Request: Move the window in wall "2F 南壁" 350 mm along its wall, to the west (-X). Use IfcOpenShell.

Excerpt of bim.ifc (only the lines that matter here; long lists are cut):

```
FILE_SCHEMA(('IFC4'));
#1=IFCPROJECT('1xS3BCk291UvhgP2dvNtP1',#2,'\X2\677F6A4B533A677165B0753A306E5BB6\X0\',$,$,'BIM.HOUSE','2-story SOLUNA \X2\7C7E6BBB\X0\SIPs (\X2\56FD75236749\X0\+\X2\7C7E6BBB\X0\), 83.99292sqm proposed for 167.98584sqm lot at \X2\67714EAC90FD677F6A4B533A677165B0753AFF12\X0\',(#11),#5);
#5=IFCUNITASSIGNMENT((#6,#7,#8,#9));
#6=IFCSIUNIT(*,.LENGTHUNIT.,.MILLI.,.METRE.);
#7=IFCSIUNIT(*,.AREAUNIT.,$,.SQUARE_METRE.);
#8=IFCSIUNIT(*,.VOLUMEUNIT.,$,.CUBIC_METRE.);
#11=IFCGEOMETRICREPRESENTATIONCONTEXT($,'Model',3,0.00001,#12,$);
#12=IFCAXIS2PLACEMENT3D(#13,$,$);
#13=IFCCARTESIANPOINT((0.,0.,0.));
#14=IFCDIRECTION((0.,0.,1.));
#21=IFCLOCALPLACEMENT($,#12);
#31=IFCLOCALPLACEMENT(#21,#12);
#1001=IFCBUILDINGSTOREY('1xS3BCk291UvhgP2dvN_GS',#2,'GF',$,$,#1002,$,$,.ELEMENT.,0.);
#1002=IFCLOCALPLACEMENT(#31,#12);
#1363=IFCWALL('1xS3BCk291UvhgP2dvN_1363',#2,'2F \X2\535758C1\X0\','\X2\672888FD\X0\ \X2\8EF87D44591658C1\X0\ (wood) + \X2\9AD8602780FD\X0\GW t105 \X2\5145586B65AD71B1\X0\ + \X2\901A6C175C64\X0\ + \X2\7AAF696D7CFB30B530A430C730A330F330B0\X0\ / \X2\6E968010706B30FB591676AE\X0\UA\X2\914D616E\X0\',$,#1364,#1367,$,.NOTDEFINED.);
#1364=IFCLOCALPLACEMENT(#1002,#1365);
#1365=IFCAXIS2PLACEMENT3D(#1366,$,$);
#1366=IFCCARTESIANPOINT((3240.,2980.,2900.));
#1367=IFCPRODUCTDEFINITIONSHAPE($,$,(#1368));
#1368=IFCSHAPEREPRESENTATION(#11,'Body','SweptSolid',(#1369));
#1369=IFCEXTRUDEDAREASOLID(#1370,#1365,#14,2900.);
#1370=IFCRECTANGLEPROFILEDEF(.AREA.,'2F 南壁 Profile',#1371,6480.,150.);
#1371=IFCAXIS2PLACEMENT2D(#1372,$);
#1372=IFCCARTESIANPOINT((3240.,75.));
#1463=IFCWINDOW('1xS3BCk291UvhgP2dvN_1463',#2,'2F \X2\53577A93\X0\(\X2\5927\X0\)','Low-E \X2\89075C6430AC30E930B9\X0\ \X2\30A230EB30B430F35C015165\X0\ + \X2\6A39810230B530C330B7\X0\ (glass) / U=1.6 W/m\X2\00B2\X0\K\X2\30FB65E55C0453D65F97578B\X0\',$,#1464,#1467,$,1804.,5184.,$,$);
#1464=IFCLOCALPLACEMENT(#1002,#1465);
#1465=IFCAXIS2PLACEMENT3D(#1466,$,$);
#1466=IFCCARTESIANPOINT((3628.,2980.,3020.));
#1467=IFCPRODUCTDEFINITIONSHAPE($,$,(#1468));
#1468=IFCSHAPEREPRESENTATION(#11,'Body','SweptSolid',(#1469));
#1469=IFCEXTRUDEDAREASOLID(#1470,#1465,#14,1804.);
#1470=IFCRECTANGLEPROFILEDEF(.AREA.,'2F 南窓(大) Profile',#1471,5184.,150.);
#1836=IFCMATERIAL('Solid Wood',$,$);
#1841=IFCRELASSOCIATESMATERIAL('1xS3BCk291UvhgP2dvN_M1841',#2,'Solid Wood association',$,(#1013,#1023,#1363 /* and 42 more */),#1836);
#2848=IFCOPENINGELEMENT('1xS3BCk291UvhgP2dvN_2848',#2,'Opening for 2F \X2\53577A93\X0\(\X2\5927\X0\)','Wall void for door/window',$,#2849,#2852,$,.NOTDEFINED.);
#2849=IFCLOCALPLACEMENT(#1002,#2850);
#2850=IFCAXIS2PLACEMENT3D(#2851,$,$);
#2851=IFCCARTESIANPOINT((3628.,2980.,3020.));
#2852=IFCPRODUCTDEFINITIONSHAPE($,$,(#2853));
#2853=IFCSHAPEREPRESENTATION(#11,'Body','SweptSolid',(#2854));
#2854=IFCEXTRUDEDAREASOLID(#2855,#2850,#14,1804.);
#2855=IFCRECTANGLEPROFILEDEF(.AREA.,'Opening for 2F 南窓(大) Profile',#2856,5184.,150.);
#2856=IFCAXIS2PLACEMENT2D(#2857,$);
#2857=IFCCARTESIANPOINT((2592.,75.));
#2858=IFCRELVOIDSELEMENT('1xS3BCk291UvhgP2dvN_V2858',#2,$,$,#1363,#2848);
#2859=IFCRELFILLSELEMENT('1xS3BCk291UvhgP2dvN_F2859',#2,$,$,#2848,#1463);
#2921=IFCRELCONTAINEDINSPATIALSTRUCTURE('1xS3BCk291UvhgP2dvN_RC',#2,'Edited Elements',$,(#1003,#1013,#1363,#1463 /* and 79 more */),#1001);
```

```python
import ifcopenshell
import ifcopenshell.api.geometry
import ifcopenshell.util.placement
import ifcopenshell.util.unit

model = ifcopenshell.open("bim.ifc")
unit_scale = ifcopenshell.util.unit.calculate_unit_scale(model)

window = model.by_guid("1xS3BCk291UvhgP2dvN_1463")
opening = window.FillsVoids[0].RelatingOpeningElement
wall = opening.VoidsElements[0].RelatingBuildingElement

wall_matrix = ifcopenshell.util.placement.get_local_placement(wall.ObjectPlacement)
shift = wall_matrix[:3, 0] * -0.35 / unit_scale
before = ifcopenshell.util.placement.get_local_placement(window.ObjectPlacement)[:3, 3].copy()

# The window is not placed relative to its opening, so move both.
for product in (opening, window):
    matrix = ifcopenshell.util.placement.get_local_placement(product.ObjectPlacement)
    matrix[:3, 3] += shift
    ifcopenshell.api.geometry.edit_object_placement(model, product=product, matrix=matrix, is_si=False)

after = ifcopenshell.util.placement.get_local_placement(window.ObjectPlacement)[:3, 3]
print("window moved by", (after - before).round(3) + 0.0)

model.write("bim_updated.ifc")
```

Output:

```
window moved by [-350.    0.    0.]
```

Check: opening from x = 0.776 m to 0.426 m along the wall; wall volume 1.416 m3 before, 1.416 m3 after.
